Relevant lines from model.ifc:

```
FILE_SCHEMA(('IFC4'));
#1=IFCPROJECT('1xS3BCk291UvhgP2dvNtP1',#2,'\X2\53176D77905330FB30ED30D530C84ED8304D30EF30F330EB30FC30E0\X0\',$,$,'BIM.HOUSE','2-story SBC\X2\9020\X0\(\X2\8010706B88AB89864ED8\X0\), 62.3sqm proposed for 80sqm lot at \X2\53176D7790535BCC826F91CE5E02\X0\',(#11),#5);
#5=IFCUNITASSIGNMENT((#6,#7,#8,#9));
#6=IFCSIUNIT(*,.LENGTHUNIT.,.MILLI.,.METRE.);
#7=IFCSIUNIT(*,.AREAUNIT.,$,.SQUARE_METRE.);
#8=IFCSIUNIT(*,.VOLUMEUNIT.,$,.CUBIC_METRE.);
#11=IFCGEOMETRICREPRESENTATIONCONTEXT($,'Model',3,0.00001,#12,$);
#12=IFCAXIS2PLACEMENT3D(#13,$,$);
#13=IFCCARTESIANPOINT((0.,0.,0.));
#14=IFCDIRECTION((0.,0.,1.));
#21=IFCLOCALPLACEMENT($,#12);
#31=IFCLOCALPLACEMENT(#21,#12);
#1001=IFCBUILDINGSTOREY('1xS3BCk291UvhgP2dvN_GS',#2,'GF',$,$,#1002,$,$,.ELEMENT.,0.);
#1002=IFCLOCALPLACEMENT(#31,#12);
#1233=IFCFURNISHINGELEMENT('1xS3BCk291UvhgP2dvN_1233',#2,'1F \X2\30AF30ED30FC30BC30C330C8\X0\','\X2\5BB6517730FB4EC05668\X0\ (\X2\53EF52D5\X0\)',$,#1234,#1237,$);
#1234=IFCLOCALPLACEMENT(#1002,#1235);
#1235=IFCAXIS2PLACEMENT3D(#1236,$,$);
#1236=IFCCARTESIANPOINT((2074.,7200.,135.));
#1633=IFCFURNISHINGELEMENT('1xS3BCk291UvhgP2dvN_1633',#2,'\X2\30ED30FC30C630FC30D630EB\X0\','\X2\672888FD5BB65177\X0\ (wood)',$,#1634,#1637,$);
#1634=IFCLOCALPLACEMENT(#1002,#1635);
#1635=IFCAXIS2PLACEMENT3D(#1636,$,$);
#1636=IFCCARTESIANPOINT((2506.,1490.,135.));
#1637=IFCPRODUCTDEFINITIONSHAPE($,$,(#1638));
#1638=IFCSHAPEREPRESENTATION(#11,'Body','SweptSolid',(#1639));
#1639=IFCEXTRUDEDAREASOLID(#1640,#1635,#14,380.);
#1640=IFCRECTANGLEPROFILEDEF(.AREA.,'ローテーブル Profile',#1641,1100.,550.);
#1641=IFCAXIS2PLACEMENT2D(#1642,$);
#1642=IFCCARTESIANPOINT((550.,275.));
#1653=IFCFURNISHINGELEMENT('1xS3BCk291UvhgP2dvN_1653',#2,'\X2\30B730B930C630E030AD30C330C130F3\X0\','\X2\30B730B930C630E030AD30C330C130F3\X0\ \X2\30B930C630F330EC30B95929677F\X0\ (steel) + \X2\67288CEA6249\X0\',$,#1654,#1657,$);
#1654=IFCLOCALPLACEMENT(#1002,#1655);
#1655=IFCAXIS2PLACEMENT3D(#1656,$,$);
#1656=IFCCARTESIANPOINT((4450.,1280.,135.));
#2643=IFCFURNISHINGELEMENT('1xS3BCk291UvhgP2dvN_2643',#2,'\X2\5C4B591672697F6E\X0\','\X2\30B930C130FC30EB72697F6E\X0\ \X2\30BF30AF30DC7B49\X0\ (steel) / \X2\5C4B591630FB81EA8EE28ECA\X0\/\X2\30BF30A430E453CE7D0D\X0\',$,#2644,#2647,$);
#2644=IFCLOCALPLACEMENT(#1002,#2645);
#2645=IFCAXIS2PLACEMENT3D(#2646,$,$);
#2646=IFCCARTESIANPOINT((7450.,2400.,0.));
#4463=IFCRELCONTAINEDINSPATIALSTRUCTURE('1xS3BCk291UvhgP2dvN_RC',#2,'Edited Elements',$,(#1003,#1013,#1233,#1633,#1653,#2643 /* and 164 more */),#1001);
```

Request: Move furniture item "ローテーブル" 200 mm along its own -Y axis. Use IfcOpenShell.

```python
import ifcopenshell
import ifcopenshell.api.geometry
import ifcopenshell.util.placement
import ifcopenshell.util.unit

model = ifcopenshell.open("model.ifc")
unit_scale = ifcopenshell.util.unit.calculate_unit_scale(model)

item = model.by_id(1633)
matrix = ifcopenshell.util.placement.get_local_placement(item.ObjectPlacement)
matrix[:3, 3] -= matrix[:3, 1] * 0.2 / unit_scale
ifcopenshell.api.geometry.edit_object_placement(model, product=item, matrix=matrix, is_si=False)

print(ifcopenshell.util.placement.get_local_placement(item.ObjectPlacement).round(3) + 0.0)

model.write("model_updated.ifc")
```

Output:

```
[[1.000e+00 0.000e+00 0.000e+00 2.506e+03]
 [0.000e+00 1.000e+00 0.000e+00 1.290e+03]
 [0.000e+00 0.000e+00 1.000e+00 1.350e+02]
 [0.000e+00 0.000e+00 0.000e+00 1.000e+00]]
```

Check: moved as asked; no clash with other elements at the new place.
